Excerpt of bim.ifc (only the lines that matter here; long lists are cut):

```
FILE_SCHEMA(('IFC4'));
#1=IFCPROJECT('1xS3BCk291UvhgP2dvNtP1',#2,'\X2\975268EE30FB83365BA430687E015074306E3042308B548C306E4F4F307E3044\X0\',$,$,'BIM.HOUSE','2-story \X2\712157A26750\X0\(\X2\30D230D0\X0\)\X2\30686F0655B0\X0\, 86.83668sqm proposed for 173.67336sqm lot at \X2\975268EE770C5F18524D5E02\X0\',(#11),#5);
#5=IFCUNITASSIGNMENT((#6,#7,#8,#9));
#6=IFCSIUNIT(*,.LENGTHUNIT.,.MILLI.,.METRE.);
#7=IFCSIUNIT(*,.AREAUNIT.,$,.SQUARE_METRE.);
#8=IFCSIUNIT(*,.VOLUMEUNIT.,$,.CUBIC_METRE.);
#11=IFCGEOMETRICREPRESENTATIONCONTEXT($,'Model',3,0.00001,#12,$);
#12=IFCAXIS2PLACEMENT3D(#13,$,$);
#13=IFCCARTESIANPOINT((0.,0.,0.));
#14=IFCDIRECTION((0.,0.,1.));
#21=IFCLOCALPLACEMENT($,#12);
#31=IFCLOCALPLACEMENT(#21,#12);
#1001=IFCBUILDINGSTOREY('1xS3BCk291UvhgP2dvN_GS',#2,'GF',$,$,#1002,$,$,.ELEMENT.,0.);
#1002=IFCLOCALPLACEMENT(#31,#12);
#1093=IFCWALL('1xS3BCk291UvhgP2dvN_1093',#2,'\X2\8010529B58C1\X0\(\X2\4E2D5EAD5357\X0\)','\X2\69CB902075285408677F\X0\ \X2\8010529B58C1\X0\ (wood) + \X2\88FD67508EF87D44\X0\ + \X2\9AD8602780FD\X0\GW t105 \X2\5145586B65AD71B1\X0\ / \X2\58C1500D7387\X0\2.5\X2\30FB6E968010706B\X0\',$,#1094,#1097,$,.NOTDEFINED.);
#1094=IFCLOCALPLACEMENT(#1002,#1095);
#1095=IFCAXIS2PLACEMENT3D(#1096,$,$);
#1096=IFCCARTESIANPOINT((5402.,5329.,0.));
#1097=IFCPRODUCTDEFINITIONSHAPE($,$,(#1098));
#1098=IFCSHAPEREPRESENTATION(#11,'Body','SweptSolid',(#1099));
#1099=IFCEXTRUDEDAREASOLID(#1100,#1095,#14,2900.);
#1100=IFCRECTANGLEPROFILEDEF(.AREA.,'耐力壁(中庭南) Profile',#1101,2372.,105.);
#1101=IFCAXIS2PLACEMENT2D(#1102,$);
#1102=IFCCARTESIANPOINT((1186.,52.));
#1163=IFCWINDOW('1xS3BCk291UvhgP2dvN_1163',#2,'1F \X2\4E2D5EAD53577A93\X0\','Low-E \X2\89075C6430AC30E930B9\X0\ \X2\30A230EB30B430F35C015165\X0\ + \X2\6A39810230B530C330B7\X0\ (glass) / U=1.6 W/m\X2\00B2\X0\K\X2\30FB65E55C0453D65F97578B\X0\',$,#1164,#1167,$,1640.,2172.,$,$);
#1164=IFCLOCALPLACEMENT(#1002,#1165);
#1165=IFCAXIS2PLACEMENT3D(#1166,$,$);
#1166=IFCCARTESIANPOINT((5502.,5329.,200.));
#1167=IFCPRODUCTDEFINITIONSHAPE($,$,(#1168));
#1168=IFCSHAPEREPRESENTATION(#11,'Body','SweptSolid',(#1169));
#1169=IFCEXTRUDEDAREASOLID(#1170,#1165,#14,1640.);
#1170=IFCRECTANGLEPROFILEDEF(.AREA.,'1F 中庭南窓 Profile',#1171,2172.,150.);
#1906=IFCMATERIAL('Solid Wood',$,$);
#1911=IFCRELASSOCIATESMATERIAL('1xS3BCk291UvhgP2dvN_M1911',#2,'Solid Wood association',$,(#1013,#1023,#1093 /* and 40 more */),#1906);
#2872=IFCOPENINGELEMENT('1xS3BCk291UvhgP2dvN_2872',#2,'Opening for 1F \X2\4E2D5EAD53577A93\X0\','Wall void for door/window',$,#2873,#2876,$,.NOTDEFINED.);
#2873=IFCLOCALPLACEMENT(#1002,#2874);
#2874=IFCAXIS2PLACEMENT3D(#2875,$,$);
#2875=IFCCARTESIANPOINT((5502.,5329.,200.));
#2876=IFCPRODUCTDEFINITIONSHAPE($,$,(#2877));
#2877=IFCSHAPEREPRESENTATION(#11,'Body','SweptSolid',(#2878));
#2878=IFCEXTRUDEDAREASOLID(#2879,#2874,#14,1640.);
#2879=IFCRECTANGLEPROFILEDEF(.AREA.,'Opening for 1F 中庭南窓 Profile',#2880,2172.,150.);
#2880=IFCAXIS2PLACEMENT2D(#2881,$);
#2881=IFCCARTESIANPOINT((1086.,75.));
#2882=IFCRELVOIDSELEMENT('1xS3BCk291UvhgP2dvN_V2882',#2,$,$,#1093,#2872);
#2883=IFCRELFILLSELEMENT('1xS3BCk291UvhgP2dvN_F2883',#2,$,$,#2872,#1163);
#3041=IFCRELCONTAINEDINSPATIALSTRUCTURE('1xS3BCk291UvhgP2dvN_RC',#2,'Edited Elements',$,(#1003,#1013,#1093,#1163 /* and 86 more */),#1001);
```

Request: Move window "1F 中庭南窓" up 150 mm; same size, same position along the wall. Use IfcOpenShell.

```python
import numpy as np
import ifcopenshell
import ifcopenshell.api.geometry
import ifcopenshell.util.placement
import ifcopenshell.util.unit

model = ifcopenshell.open("bim.ifc")
unit_scale = ifcopenshell.util.unit.calculate_unit_scale(model)

window = model.by_guid("1xS3BCk291UvhgP2dvN_1163")
opening = window.FillsVoids[0].RelatingOpeningElement
dz = 150.0

shift = np.array([0.0, 0.0, dz])
# The window is not placed relative to its opening, so move both.
for product in (opening, window):
    matrix = ifcopenshell.util.placement.get_local_placement(product.ObjectPlacement)
    matrix[:3, 3] += shift
    ifcopenshell.api.geometry.edit_object_placement(model, product=product, matrix=matrix, is_si=False)

print(f"moved by {dz * unit_scale:+.3f} m")

model.write("bim_edited.ifc")
```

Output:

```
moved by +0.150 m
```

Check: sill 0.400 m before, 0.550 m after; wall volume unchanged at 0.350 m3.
